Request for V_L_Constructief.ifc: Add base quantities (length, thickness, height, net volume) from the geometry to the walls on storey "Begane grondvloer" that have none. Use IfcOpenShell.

First a look at what the model holds.

```python
import ifcopenshell
import ifcopenshell.util.element
import ifcopenshell.util.unit

model = ifcopenshell.open("V_L_Constructief.ifc")
print(model.schema)
for unit_type in ("LENGTHUNIT", "AREAUNIT", "VOLUMEUNIT"):
    print(unit_type, ifcopenshell.util.unit.calculate_unit_scale(model, unit_type))
storey = next(s for s in model.by_type("IfcBuildingStorey") if s.Name == "Begane grondvloer")
walls = [e for e in ifcopenshell.util.element.get_decomposition(storey) if e.is_a("IfcWall")]
for e in sorted(walls, key=lambda e: e.id()):
    print(e.id(), e.is_a(), e.Name, list(ifcopenshell.util.element.get_psets(e, qtos_only=True)), sep=" | ")
```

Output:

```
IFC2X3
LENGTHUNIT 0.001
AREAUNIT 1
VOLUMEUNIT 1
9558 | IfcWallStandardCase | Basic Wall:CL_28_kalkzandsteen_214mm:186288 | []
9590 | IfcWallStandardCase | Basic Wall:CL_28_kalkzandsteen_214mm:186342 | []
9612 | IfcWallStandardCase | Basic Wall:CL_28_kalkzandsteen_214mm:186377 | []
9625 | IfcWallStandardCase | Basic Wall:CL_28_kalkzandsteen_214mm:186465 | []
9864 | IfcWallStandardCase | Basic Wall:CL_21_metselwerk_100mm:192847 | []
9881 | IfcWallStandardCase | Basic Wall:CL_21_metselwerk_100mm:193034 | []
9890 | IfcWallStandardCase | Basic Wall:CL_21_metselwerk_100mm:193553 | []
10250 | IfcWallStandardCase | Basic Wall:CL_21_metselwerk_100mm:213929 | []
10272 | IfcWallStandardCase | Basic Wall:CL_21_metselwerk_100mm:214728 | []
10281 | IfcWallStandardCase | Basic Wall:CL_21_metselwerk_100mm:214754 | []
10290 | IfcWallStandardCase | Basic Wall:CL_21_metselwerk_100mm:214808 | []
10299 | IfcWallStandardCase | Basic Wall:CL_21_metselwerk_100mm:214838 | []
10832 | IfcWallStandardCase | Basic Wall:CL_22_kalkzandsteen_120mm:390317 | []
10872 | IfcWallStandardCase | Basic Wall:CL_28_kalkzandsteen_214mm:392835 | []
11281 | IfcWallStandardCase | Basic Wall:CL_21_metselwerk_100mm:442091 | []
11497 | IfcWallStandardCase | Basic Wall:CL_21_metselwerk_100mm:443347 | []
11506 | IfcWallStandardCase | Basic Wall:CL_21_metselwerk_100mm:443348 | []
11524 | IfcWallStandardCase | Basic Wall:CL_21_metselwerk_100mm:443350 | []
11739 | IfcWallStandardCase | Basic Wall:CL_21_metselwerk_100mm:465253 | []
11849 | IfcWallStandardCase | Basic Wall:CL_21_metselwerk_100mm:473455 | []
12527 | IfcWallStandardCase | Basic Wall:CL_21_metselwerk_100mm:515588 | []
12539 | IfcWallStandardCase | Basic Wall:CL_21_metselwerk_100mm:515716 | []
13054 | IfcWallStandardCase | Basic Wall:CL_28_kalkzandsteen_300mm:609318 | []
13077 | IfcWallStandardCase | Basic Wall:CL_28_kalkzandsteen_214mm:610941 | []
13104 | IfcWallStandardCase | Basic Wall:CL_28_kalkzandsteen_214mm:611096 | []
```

```python
import ifcopenshell
import ifcopenshell.api.pset
import ifcopenshell.geom
import ifcopenshell.util.element
import ifcopenshell.util.shape
import ifcopenshell.util.unit

model = ifcopenshell.open("V_L_Constructief.ifc")
unit_scale = ifcopenshell.util.unit.calculate_unit_scale(model)
volume_scale = ifcopenshell.util.unit.calculate_unit_scale(model, "VOLUMEUNIT")
settings = ifcopenshell.geom.settings()

storey = next(s for s in model.by_type("IfcBuildingStorey") if s.Name == "Begane grondvloer")
walls = [e for e in ifcopenshell.util.element.get_decomposition(storey) if e.is_a("IfcWall")]

for e in sorted(walls, key=lambda e: e.id()):
    if ifcopenshell.util.element.get_psets(e, qtos_only=True, should_inherit=False):
        continue
    # Geometry comes back in metres, in the element's own axes.
    shape = ifcopenshell.geom.create_shape(settings, e)
    values = {
        "Length": ifcopenshell.util.shape.get_x(shape.geometry) / unit_scale,
        "Width": ifcopenshell.util.shape.get_y(shape.geometry) / unit_scale,
        "Height": ifcopenshell.util.shape.get_z(shape.geometry) / unit_scale,
        "NetVolume": ifcopenshell.util.shape.get_volume(shape.geometry) / volume_scale,
    }
    qto = ifcopenshell.api.pset.add_qto(model, product=e, name="BaseQuantities")
    ifcopenshell.api.pset.edit_qto(model, qto=qto, properties=values)
    print(e.id(), {k: round(v, 3) for k, v in values.items()})

model.write("V_L_Constructief-out.ifc")
```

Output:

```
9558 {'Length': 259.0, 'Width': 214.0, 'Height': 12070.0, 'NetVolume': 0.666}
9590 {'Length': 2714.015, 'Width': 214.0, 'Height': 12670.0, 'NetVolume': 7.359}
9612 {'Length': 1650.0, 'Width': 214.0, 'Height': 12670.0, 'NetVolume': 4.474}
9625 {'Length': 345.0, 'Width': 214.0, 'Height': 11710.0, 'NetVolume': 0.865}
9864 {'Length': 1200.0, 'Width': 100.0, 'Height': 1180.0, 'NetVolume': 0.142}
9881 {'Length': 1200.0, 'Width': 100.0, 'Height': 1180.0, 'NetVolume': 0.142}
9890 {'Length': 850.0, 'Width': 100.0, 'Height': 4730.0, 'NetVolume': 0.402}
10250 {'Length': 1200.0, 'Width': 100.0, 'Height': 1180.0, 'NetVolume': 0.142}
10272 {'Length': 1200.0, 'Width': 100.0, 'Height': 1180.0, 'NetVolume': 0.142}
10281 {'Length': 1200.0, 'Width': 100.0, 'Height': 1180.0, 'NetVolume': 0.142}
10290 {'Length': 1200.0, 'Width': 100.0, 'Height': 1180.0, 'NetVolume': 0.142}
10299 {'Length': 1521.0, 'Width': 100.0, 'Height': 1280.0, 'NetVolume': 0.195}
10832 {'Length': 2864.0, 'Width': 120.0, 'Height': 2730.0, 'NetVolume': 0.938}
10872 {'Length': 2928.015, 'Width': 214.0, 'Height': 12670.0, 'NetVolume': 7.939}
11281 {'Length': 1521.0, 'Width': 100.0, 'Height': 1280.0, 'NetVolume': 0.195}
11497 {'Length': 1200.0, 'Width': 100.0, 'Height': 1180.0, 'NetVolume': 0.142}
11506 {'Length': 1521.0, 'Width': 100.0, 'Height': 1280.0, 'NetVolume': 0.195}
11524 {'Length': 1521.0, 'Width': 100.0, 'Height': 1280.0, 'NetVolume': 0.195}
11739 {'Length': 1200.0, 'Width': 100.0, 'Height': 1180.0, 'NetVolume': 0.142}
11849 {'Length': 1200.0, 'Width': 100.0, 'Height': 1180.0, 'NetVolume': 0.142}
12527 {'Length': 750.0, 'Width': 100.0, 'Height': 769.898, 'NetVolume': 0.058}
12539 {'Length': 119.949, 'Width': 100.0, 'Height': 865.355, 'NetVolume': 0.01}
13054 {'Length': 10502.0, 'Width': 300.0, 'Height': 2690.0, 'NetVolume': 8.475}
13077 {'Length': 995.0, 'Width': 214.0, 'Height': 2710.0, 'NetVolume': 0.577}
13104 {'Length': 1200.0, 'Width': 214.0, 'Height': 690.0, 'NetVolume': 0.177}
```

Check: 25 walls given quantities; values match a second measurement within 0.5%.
